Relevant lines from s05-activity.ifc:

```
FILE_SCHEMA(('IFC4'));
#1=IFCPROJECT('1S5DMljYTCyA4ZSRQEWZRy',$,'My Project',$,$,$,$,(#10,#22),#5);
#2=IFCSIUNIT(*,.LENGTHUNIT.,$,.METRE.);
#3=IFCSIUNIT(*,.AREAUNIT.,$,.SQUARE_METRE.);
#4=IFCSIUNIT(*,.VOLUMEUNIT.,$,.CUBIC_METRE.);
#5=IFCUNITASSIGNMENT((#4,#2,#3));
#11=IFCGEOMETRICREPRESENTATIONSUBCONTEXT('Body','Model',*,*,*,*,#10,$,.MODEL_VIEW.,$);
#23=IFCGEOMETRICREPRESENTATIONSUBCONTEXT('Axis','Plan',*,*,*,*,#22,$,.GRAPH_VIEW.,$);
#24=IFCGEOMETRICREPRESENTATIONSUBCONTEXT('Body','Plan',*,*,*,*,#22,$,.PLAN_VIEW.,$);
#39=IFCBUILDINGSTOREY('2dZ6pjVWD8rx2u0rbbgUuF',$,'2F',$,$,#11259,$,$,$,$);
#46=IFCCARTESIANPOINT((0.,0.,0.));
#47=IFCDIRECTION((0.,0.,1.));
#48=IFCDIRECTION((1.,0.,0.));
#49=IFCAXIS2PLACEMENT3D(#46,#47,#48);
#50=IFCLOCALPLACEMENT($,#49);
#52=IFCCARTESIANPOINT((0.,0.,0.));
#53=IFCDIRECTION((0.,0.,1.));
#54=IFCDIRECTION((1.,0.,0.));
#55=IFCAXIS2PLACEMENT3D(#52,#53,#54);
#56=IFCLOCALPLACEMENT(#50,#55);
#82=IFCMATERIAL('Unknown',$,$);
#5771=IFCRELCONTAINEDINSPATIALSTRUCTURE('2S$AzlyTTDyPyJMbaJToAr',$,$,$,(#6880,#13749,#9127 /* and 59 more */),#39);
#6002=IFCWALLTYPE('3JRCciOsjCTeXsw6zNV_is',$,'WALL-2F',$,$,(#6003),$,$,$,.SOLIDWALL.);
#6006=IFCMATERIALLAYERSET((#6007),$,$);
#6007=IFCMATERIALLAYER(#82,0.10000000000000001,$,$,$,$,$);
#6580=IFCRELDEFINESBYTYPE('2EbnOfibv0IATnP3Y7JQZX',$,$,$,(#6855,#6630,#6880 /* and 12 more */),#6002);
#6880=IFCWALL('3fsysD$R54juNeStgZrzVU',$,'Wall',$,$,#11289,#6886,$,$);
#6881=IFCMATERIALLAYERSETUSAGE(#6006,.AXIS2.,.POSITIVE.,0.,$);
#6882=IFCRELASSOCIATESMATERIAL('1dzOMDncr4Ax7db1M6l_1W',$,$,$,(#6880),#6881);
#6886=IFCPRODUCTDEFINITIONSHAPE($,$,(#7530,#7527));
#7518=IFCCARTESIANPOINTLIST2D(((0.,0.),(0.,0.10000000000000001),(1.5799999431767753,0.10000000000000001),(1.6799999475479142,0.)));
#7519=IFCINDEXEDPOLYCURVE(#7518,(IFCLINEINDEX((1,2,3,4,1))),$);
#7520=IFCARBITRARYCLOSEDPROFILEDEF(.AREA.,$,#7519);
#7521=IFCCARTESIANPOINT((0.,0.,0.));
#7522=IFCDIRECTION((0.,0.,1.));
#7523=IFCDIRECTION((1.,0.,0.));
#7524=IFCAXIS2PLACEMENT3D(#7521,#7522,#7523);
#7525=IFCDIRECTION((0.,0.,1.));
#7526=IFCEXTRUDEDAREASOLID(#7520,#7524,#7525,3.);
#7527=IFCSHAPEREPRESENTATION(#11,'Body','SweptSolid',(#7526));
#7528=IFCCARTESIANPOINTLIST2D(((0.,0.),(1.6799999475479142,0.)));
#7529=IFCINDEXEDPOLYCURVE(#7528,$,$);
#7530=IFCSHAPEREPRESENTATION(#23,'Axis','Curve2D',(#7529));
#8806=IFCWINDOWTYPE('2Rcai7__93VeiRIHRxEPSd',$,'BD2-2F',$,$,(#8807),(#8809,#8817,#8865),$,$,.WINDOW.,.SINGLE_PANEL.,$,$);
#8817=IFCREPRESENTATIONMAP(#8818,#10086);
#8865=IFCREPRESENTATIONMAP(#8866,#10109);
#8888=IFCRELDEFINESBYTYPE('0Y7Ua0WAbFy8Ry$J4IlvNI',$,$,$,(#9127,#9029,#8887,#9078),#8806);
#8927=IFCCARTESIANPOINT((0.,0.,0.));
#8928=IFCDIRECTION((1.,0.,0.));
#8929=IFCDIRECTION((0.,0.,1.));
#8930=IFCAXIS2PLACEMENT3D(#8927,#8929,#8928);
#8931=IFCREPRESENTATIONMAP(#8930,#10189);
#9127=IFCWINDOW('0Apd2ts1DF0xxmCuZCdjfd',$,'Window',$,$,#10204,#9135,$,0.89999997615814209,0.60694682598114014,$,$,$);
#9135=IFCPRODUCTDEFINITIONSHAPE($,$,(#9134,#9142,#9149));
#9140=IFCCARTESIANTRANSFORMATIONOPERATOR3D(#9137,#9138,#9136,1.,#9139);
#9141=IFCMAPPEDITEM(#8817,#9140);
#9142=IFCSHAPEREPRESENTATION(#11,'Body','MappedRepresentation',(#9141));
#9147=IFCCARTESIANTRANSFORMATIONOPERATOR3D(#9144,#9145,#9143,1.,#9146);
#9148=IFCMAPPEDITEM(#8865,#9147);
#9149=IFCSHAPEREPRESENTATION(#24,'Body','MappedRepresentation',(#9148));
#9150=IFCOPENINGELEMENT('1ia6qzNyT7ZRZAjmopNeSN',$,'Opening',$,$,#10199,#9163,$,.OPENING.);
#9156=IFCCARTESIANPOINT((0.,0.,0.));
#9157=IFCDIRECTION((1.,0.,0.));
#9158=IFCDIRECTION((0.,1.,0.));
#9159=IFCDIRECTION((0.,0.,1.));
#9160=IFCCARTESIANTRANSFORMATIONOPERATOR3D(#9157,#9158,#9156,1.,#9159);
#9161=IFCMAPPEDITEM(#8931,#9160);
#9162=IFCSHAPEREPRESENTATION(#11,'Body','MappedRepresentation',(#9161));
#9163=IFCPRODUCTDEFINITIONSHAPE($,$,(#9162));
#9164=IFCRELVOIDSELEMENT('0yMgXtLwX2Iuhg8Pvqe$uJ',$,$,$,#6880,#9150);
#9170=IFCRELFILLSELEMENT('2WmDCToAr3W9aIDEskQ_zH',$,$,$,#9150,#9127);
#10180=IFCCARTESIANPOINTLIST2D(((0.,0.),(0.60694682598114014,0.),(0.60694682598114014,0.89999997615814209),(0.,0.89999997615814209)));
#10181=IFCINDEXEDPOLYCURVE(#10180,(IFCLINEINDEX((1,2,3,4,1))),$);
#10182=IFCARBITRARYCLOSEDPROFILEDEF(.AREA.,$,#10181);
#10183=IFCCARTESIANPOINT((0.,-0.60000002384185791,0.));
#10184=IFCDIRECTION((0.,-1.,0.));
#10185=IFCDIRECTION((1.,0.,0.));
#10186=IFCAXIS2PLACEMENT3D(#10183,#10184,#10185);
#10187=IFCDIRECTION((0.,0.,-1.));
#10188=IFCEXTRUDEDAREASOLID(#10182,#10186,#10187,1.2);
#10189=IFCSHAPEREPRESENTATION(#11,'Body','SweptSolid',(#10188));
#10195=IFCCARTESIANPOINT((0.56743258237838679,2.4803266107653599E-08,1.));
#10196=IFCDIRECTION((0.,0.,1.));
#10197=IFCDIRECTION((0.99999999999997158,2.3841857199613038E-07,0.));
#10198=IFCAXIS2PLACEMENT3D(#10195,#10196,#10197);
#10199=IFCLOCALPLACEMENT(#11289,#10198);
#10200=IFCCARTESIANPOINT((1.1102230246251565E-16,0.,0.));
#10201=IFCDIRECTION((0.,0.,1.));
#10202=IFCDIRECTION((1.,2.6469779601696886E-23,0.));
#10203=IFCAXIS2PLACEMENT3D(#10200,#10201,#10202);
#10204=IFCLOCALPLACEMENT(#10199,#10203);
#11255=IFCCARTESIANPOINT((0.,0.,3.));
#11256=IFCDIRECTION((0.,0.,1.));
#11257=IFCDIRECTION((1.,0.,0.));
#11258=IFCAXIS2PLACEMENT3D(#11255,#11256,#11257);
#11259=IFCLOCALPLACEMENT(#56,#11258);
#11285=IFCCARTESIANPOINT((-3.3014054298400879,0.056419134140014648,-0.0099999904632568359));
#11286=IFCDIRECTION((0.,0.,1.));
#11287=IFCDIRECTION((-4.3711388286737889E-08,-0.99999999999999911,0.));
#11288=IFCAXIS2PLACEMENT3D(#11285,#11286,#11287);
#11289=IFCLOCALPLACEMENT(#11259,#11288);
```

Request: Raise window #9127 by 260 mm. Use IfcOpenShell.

```python
import numpy as np
import ifcopenshell
import ifcopenshell.api.geometry
import ifcopenshell.util.placement
import ifcopenshell.util.unit

model = ifcopenshell.open("s05-activity.ifc")
unit_scale = ifcopenshell.util.unit.calculate_unit_scale(model)

window = model.by_guid("0Apd2ts1DF0xxmCuZCdjfd")
opening = window.FillsVoids[0].RelatingOpeningElement
dz = 0.26 / unit_scale

shift = np.array([0.0, 0.0, dz])
# The window is placed relative to its opening, so it follows when the opening moves.
matrix = ifcopenshell.util.placement.get_local_placement(opening.ObjectPlacement)
matrix[:3, 3] += shift
ifcopenshell.api.geometry.edit_object_placement(
    model, product=opening, matrix=matrix, is_si=False, should_transform_children=True
)

print(f"moved by {dz * unit_scale:+.3f} m")

model.write("s05-activity_v2.ifc")
```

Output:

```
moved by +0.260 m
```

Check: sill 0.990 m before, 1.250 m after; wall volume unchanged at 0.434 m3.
